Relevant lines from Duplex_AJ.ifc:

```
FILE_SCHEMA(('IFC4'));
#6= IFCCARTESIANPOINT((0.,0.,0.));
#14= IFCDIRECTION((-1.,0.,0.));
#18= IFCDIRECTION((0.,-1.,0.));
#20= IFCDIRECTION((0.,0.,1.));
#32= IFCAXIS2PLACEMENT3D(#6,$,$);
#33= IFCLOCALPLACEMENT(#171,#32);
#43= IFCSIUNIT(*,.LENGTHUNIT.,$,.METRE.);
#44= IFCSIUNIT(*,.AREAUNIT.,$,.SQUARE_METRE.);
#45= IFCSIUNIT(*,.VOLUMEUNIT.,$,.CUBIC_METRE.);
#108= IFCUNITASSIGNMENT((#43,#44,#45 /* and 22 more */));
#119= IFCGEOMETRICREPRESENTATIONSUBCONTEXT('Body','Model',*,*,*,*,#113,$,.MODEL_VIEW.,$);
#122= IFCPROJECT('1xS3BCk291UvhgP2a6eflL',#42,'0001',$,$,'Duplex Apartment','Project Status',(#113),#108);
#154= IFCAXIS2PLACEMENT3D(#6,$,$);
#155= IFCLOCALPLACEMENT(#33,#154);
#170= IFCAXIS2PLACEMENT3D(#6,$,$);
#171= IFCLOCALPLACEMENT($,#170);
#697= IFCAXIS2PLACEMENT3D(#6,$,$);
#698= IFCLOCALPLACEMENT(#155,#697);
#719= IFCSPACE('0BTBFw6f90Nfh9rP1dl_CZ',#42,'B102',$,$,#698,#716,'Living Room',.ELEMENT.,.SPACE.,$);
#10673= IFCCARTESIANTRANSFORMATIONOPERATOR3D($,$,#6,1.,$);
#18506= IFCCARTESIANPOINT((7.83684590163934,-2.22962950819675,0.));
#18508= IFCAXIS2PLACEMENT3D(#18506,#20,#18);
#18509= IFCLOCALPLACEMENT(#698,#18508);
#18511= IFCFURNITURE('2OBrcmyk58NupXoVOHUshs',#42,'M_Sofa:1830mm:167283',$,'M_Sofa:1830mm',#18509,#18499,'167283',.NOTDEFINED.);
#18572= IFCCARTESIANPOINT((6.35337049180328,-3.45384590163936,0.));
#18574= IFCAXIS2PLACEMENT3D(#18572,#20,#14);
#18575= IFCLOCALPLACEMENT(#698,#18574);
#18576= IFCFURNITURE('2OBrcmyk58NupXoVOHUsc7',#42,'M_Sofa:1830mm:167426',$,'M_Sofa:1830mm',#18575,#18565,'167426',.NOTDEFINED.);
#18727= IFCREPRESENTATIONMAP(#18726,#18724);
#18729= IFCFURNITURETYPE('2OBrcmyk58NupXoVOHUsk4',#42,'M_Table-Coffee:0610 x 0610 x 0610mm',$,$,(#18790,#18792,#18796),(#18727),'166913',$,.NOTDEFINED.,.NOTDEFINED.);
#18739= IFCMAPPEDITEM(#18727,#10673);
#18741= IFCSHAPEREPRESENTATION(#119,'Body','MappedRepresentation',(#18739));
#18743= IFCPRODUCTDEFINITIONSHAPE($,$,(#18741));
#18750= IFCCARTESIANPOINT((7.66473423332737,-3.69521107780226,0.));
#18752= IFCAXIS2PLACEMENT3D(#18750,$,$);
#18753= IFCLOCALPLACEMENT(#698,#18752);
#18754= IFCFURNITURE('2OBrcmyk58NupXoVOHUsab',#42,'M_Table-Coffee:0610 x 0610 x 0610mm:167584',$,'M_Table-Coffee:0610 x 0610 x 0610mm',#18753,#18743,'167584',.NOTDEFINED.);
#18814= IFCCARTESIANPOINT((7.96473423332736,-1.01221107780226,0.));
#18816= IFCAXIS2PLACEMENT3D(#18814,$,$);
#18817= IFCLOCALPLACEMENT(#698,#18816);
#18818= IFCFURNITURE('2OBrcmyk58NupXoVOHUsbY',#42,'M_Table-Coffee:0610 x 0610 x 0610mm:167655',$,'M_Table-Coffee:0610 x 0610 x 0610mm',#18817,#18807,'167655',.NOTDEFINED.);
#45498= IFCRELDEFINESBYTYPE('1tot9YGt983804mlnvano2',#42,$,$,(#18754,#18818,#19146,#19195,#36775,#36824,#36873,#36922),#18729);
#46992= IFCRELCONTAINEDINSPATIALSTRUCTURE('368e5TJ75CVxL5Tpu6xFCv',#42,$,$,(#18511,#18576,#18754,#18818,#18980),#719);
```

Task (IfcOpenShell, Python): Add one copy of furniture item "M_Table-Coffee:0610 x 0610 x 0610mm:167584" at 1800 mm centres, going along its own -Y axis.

```python
import ifcopenshell
import ifcopenshell.api.geometry
import ifcopenshell.api.root
import ifcopenshell.util.element
import ifcopenshell.util.placement

model = ifcopenshell.open("Duplex_AJ.ifc")


def reuse_history(source, copy):
    """copy_class also copies each property set's owner history, people and application; keep the originals."""
    for rel in copy.IsDefinedBy:
        if rel.is_a("IfcRelDefinesByProperties") and (history := rel.RelatingPropertyDefinition.OwnerHistory):
            rel.RelatingPropertyDefinition.OwnerHistory = source.OwnerHistory
            ifcopenshell.util.element.remove_deep2(model, history)


source = model.by_guid("2OBrcmyk58NupXoVOHUsab")
base = ifcopenshell.util.placement.get_local_placement(source.ObjectPlacement)
step = -base[:3, 1] * 1.8

for i in range(1, 2):
    copy = ifcopenshell.api.root.copy_class(model, product=source)
    copy.Representation = ifcopenshell.util.element.copy_deep(
        model, source.Representation, exclude=["IfcGeometricRepresentationContext", "IfcRepresentationMap"]
    )
    copy.Name = "M_Table-Coffee:0610 x 0610 x 0610mm"
    copy.Tag = None
    reuse_history(source, copy)
    matrix = base.copy()
    matrix[:3, 3] += i * step
    print("added at", matrix[:3, 3].round(3) + 0.0)
    ifcopenshell.api.geometry.edit_object_placement(model, product=copy, matrix=matrix, is_si=False)

model.write("Duplex_AJ_v2.ifc")
```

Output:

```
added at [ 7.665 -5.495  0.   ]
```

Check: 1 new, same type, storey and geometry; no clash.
